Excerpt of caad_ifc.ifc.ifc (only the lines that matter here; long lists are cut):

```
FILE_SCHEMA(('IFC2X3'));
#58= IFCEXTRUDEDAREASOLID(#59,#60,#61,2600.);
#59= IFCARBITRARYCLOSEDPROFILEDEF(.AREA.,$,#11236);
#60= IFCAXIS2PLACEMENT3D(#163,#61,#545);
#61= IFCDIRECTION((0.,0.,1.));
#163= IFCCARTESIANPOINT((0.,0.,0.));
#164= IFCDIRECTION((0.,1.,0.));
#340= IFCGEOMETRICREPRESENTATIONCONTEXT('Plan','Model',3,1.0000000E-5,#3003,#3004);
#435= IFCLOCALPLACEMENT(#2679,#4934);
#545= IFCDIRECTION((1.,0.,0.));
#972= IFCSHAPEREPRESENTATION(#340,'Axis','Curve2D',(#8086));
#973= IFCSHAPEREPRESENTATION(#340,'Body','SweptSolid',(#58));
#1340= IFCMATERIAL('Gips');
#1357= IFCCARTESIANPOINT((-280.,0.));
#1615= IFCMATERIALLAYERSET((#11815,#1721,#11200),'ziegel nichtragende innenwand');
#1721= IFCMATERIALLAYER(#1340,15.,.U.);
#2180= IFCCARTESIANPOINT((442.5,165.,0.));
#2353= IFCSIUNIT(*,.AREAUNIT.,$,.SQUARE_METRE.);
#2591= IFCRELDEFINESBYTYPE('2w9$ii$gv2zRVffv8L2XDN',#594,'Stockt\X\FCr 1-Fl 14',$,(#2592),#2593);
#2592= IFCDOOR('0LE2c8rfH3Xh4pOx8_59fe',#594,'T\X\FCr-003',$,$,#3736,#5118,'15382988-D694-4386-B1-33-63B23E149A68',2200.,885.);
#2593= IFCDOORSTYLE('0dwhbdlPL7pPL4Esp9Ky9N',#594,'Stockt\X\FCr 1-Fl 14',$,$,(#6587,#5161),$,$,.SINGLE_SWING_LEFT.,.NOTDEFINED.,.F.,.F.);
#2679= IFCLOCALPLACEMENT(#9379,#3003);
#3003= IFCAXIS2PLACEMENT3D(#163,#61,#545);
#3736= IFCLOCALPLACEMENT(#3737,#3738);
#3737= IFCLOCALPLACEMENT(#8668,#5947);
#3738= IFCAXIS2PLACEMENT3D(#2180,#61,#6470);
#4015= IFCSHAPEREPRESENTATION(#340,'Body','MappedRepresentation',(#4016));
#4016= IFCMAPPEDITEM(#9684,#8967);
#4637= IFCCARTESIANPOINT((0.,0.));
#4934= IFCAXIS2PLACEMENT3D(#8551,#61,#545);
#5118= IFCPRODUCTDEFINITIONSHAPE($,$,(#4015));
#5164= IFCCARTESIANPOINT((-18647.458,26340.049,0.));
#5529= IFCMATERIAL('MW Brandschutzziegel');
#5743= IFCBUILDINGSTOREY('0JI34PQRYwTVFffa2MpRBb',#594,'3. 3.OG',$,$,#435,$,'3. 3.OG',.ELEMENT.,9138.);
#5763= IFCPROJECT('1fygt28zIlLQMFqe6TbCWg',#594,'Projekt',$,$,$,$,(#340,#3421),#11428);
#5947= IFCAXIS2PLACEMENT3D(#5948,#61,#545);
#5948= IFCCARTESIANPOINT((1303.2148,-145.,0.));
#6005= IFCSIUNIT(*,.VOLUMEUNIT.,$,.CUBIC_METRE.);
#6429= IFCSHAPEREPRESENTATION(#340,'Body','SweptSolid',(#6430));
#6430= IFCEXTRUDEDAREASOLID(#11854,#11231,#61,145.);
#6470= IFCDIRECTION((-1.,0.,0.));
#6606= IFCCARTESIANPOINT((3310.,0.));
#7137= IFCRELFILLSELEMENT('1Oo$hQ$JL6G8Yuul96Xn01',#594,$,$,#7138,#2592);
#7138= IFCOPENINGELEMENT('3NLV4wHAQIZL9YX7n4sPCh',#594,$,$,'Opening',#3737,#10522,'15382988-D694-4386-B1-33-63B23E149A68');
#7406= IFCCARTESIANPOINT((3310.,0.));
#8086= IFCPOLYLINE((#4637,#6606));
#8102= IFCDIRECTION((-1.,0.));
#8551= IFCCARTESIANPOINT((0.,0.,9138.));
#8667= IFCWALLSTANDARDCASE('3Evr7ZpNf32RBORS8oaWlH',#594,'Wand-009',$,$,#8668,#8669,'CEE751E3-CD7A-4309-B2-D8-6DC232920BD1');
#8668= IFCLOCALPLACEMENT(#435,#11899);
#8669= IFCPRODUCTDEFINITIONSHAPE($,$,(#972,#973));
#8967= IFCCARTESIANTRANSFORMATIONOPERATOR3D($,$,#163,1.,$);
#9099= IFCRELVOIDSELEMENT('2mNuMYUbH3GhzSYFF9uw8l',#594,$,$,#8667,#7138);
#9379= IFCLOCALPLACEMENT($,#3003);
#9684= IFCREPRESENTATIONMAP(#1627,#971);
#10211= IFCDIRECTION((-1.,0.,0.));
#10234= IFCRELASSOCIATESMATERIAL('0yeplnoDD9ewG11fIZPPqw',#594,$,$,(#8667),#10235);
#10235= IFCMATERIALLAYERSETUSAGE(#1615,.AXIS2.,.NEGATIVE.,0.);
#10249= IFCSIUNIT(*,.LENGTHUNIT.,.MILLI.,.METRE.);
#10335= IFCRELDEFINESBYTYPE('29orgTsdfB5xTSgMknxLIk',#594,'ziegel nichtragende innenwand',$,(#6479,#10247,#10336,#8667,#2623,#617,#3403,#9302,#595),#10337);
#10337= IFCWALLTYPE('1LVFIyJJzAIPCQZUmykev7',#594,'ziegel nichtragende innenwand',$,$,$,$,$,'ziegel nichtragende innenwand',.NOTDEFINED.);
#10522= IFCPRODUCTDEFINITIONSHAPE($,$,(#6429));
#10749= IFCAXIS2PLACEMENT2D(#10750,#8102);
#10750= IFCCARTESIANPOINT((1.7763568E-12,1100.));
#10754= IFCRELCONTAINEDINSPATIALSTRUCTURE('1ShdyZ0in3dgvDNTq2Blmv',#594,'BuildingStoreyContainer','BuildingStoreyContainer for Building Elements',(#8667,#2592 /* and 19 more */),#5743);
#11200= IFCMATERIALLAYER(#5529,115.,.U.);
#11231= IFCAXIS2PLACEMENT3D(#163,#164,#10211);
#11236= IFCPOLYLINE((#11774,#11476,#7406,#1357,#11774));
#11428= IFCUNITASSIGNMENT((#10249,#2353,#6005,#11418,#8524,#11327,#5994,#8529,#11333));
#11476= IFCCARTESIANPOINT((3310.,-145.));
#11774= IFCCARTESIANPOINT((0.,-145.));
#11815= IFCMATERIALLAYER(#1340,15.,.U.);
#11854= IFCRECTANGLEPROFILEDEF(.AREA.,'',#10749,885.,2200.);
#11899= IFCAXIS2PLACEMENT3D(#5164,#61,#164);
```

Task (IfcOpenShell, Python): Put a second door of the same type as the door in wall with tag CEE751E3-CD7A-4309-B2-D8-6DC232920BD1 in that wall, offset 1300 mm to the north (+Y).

```python
import ifcopenshell
import ifcopenshell.api.feature
import ifcopenshell.api.geometry
import ifcopenshell.api.root
import ifcopenshell.geom
import ifcopenshell.util.element
import ifcopenshell.util.placement
import ifcopenshell.util.shape

model = ifcopenshell.open("caad_ifc.ifc.ifc")
settings = ifcopenshell.geom.settings()


def volume(element):
    """Net volume in cubic metres, openings subtracted."""
    shape = ifcopenshell.geom.create_shape(settings, element)
    return ifcopenshell.util.shape.get_volume(shape.geometry)


door = model.by_guid("0LE2c8rfH3Xh4pOx8_59fe")
opening = door.FillsVoids[0].RelatingOpeningElement
wall = opening.VoidsElements[0].RelatingBuildingElement
before = volume(wall)
shift = ifcopenshell.util.placement.get_local_placement(wall.ObjectPlacement)[:3, 0] * 1300.0

# copy_class copies the void relationship, type, container and properties, but no geometry.
new_opening = ifcopenshell.api.root.copy_class(model, product=opening)
new_opening.Representation = ifcopenshell.util.element.copy_deep(
    model, opening.Representation, exclude=["IfcGeometricRepresentationContext", "IfcRepresentationMap"]
)
new_opening.Tag = None
new_door = ifcopenshell.api.root.copy_class(model, product=door)
new_door.Representation = ifcopenshell.util.element.copy_deep(
    model, door.Representation, exclude=["IfcGeometricRepresentationContext", "IfcRepresentationMap"]
)
new_door.Tag = None
fills = ifcopenshell.api.feature.add_filling(model, opening=new_opening, element=new_door)
fills.OwnerHistory = new_door.OwnerHistory  # required in IFC2X3

for old, new in ((opening, new_opening), (door, new_door)):
    matrix = ifcopenshell.util.placement.get_local_placement(old.ObjectPlacement)
    matrix[:3, 3] += shift
    ifcopenshell.api.geometry.edit_object_placement(model, product=new, matrix=matrix, is_si=False)

after = volume(wall)

print(f"wall volume {before:.3f} -> {after:.3f} m3")

model.write("caad_ifc.ifc_rev.ifc")
```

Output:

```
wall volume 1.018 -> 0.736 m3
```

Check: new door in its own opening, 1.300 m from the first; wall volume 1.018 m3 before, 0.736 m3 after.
